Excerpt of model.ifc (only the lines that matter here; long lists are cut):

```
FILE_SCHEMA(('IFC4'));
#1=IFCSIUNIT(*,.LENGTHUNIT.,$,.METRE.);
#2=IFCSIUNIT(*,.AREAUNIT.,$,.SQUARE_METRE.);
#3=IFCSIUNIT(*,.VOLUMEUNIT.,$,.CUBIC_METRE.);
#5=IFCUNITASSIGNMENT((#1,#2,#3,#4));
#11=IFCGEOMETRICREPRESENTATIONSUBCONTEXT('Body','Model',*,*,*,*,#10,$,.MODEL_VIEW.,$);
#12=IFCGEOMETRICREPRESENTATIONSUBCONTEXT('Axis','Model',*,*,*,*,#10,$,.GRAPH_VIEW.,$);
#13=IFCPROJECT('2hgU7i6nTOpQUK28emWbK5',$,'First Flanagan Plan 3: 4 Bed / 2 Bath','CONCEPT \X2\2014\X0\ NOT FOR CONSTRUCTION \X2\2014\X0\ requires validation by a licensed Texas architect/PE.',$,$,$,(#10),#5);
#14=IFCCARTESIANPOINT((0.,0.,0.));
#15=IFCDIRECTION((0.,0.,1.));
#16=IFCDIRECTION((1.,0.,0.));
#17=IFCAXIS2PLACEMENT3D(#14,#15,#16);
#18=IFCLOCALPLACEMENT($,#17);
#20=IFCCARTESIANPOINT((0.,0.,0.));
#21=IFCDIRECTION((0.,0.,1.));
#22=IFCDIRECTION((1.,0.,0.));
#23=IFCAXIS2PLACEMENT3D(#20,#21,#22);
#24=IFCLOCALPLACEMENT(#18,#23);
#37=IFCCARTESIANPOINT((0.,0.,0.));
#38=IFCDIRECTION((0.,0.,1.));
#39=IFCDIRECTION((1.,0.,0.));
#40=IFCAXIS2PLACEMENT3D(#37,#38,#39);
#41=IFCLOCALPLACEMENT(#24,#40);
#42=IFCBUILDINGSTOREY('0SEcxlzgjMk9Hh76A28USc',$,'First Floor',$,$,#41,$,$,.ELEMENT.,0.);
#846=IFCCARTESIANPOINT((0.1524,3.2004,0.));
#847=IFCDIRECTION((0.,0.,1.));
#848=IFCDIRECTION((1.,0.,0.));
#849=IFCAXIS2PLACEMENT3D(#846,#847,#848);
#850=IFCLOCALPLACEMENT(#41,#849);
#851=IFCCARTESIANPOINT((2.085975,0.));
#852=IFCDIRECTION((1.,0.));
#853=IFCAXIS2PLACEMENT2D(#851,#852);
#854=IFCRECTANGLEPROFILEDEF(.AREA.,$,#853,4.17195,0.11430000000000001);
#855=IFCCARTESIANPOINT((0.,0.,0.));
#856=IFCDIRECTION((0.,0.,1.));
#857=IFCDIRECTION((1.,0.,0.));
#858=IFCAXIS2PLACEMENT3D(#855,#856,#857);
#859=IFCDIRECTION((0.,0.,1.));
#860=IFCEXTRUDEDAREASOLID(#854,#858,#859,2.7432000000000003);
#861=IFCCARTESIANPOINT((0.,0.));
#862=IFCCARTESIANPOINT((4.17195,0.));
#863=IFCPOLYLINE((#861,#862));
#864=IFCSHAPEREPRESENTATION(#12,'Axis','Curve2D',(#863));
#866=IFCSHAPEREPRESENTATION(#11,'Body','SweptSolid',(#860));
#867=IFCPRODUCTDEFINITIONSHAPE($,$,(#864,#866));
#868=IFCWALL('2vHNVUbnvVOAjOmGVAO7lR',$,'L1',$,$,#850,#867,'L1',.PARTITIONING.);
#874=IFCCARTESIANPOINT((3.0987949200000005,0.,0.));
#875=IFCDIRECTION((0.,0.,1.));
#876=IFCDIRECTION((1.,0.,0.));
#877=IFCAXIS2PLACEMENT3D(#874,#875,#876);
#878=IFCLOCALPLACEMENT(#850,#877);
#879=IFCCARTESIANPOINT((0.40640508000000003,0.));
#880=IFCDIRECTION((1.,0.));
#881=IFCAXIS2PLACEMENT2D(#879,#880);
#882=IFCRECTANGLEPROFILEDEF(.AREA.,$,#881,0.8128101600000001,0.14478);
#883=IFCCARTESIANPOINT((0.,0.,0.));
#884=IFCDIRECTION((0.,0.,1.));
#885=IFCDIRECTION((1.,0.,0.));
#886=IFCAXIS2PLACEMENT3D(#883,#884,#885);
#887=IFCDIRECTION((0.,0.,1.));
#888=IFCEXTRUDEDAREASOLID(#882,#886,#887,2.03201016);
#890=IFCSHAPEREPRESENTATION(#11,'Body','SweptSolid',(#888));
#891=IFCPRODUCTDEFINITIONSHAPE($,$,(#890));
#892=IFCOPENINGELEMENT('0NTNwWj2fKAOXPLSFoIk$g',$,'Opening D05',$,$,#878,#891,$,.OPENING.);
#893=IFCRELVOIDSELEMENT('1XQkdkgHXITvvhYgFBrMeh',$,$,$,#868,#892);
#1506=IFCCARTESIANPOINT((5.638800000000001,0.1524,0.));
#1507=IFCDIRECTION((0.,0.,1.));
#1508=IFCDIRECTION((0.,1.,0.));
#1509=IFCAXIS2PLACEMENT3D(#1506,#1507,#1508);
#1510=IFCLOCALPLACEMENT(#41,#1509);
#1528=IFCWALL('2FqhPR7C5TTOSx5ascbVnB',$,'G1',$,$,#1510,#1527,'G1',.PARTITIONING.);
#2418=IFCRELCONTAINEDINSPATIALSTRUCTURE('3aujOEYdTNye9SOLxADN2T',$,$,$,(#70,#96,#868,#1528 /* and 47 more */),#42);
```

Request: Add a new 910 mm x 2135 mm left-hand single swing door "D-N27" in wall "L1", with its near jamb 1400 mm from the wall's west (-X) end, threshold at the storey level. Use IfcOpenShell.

```python
import numpy as np
import ifcopenshell
import ifcopenshell.api.feature
import ifcopenshell.api.geometry
import ifcopenshell.api.root
import ifcopenshell.api.spatial
import ifcopenshell.geom
import ifcopenshell.util.element
import ifcopenshell.util.placement
import ifcopenshell.util.representation
import ifcopenshell.util.shape
import ifcopenshell.util.unit

model = ifcopenshell.open("model.ifc")
unit_scale = ifcopenshell.util.unit.calculate_unit_scale(model)
settings = ifcopenshell.geom.settings()


def volume(element):
    """Net volume in cubic metres, openings subtracted."""
    shape = ifcopenshell.geom.create_shape(settings, element)
    return ifcopenshell.util.shape.get_volume(shape.geometry)


wall = model.by_guid("2vHNVUbnvVOAjOmGVAO7lR")
storey = ifcopenshell.util.element.get_container(wall, ifc_class="IfcBuildingStorey")
context = ifcopenshell.util.representation.get_context(model, "Model", "Body", "MODEL_VIEW")
before = volume(wall)

width, height, from_end, sill = 0.91, 2.135, 1.4, 0.0  # metres

# The wall runs along its own X axis, and the end named is its -X end.
wall_shape = ifcopenshell.geom.create_shape(settings, wall)
x, y, z = ifcopenshell.util.shape.get_vertices(wall_shape.geometry).T
start = x.min() + from_end
face, thickness = float(y.min()), float(y.max() - y.min())
wall_matrix = ifcopenshell.util.placement.get_local_placement(wall.ObjectPlacement)
level = ifcopenshell.util.placement.get_local_placement(storey.ObjectPlacement)[2, 3]


def in_wall(x, y):
    """Placement at x, y metres in the wall's axes, at sill height."""
    matrix = wall_matrix.copy()
    matrix[:, 3] = wall_matrix @ np.array([x / unit_scale, y / unit_scale, 0.0, 1.0])
    matrix[2, 3] = level + sill / unit_scale
    return matrix


# Opening: a box that overshoots both wall faces by 50 mm.
opening = ifcopenshell.api.root.create_entity(model, ifc_class="IfcOpeningElement", predefined_type="OPENING")
box = ifcopenshell.api.geometry.add_wall_representation(
    model, context=context, length=width, height=height, thickness=thickness + 0.1
)
ifcopenshell.api.geometry.assign_representation(model, product=opening, representation=box)
ifcopenshell.api.geometry.edit_object_placement(model, product=opening, matrix=in_wall(start, face - 0.05), is_si=False)
ifcopenshell.api.feature.add_feature(model, feature=opening, element=wall)

door = ifcopenshell.api.root.create_entity(model, ifc_class="IfcDoor", name="D-N27", predefined_type="DOOR")
door.OverallWidth, door.OverallHeight = width / unit_scale, height / unit_scale
door.OperationType = "SINGLE_SWING_LEFT"
body = ifcopenshell.api.geometry.add_door_representation(
    model,
    context=context,
    overall_width=door.OverallWidth,
    overall_height=door.OverallHeight,
    operation_type="SINGLE_SWING_LEFT",
    lining_properties={"LiningDepth": thickness / unit_scale, "ThresholdDepth": thickness / unit_scale},
)
ifcopenshell.api.geometry.assign_representation(model, product=door, representation=body)
ifcopenshell.api.spatial.assign_container(model, products=[door], relating_structure=storey)
ifcopenshell.api.feature.add_filling(model, opening=opening, element=door)

# The lining spans the wall, so the door starts at the wall face.
ifcopenshell.api.geometry.edit_object_placement(model, product=door, matrix=in_wall(start, face), is_si=False)

after = volume(wall)

print(f"wall volume {before:.3f} -> {after:.3f} m3")

model.write("model_v2.ifc")
```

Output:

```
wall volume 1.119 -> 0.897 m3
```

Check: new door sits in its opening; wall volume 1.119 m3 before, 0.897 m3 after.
